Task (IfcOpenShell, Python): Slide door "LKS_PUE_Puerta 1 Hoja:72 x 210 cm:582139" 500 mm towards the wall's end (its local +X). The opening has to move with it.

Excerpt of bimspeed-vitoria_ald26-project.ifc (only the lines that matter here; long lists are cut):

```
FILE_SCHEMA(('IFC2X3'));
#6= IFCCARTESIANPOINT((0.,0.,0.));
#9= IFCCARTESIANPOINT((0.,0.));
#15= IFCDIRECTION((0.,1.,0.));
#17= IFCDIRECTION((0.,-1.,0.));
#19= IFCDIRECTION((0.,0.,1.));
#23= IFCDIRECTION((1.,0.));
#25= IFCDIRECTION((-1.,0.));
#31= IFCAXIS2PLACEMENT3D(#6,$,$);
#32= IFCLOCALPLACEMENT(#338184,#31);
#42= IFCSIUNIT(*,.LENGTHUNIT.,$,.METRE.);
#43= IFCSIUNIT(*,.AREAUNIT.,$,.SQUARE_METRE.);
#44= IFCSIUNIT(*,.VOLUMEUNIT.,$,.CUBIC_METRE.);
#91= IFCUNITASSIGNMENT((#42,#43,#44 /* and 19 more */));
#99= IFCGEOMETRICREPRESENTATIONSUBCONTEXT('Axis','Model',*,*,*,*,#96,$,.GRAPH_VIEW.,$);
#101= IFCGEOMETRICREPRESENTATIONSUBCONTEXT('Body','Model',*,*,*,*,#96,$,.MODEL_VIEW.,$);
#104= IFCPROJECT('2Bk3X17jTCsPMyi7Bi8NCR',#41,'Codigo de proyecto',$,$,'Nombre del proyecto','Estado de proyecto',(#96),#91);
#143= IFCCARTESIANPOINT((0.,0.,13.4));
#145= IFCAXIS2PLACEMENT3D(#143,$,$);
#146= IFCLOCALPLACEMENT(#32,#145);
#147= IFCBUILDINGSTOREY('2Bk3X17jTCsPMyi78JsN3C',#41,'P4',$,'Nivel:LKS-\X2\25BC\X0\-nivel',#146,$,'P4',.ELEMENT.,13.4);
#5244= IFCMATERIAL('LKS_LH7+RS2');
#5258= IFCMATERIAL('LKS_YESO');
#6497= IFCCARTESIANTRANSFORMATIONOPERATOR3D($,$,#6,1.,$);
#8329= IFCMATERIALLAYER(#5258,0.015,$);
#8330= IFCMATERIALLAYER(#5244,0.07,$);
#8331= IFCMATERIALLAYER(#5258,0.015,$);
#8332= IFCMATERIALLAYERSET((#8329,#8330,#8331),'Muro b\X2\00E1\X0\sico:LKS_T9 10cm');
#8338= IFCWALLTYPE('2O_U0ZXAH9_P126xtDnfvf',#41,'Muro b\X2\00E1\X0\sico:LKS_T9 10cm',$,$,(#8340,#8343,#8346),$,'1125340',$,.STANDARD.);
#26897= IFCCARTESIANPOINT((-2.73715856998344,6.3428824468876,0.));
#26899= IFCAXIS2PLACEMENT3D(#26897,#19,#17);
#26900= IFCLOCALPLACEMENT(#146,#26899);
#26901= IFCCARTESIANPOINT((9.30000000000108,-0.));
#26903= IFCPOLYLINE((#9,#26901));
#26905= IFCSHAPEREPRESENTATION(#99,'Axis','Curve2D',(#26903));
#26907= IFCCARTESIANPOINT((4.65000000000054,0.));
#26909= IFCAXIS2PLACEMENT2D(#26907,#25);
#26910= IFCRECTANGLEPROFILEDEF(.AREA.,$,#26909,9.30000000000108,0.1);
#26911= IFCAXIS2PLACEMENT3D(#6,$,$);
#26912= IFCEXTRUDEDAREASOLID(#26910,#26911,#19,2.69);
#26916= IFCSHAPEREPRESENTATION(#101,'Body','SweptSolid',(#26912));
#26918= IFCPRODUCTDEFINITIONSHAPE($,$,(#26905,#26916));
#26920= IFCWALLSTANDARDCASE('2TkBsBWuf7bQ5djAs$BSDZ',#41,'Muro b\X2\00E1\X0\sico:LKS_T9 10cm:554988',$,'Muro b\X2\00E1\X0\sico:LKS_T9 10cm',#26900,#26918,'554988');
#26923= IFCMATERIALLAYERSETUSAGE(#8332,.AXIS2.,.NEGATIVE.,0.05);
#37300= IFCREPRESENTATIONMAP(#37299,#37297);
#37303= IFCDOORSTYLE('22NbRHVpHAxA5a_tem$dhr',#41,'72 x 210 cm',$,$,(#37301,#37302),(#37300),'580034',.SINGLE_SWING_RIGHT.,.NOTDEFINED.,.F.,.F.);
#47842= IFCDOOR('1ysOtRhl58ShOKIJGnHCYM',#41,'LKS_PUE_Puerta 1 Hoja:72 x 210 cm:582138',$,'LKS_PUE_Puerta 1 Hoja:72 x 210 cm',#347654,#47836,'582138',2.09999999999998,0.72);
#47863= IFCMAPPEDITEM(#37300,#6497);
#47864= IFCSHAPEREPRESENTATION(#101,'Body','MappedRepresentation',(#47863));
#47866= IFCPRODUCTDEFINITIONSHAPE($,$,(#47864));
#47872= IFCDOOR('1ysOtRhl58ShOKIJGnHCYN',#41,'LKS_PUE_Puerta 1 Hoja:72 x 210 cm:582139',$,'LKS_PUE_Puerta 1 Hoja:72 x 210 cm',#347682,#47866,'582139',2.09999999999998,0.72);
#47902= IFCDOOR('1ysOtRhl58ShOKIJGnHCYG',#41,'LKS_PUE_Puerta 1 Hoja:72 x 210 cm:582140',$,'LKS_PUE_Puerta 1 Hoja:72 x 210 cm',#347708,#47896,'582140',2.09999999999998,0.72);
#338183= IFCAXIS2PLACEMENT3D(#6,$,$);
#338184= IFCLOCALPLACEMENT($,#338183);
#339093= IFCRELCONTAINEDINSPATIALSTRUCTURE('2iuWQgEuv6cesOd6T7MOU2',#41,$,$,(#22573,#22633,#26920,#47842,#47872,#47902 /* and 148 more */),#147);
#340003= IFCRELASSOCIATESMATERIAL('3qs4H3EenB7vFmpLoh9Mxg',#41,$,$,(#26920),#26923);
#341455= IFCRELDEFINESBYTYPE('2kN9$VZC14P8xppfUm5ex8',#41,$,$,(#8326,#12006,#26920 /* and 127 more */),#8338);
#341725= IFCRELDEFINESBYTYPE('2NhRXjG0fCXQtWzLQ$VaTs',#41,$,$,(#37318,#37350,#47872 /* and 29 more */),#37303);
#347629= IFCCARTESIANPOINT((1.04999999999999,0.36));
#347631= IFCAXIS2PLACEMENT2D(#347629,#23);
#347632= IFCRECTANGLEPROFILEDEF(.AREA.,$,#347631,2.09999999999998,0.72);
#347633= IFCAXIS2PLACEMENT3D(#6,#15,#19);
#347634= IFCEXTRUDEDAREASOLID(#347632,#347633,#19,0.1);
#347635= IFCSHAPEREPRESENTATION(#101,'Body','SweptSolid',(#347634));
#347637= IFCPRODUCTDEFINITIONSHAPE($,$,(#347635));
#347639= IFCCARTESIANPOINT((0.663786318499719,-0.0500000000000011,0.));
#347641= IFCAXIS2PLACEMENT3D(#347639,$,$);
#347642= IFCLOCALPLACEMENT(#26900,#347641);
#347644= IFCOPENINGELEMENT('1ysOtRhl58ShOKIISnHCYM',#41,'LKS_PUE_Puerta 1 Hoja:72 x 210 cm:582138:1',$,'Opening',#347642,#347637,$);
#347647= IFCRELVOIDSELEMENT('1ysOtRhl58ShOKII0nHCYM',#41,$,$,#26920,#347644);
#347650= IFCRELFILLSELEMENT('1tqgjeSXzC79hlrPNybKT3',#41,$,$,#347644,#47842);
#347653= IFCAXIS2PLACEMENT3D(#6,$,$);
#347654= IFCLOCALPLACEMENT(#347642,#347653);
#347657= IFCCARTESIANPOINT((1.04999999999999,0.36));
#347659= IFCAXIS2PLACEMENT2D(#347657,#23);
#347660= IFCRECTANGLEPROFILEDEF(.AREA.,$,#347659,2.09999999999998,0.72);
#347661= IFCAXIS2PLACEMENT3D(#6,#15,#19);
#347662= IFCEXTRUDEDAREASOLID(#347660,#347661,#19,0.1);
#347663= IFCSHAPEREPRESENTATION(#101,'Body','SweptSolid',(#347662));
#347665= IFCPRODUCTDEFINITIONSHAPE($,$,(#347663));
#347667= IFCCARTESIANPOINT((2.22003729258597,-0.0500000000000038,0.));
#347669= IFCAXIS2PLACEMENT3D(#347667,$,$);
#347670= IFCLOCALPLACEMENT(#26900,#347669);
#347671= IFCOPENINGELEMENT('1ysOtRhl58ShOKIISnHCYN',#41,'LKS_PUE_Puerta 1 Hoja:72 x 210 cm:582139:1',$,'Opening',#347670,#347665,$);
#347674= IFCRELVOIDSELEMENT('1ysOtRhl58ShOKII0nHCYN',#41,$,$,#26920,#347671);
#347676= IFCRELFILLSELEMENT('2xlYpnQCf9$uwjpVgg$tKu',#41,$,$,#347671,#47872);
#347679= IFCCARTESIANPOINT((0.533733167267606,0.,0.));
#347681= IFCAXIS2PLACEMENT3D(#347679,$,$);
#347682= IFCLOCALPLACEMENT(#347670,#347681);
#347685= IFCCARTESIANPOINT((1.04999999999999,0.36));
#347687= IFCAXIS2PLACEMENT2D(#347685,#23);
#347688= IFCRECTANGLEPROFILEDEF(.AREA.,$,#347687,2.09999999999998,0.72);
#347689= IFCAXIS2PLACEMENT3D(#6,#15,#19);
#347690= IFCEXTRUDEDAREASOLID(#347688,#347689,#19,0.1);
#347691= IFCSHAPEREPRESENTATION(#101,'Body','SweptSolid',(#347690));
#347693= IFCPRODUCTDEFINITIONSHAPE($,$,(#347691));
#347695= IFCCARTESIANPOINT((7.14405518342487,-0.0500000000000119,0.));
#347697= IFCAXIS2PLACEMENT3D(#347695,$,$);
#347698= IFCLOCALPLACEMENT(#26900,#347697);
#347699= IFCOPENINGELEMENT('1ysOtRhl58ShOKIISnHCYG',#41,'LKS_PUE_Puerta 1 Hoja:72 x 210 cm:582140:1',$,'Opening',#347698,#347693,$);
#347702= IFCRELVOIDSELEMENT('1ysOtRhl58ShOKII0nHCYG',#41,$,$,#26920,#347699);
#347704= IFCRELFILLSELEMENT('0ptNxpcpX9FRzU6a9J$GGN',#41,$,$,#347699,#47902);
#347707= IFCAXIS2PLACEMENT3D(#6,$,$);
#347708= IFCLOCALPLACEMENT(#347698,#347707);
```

```python
import ifcopenshell
import ifcopenshell.api.geometry
import ifcopenshell.util.placement
import ifcopenshell.util.unit

model = ifcopenshell.open("bimspeed-vitoria_ald26-project.ifc")
unit_scale = ifcopenshell.util.unit.calculate_unit_scale(model)

door = model.by_guid("1ysOtRhl58ShOKIJGnHCYN")
opening = door.FillsVoids[0].RelatingOpeningElement
wall = opening.VoidsElements[0].RelatingBuildingElement

wall_matrix = ifcopenshell.util.placement.get_local_placement(wall.ObjectPlacement)
shift = wall_matrix[:3, 0] * 0.5 / unit_scale
before = ifcopenshell.util.placement.get_local_placement(door.ObjectPlacement)[:3, 3].copy()

# The door is placed relative to its opening, so it follows when the opening moves.
matrix = ifcopenshell.util.placement.get_local_placement(opening.ObjectPlacement)
matrix[:3, 3] += shift
ifcopenshell.api.geometry.edit_object_placement(
    model, product=opening, matrix=matrix, is_si=False, should_transform_children=True
)

after = ifcopenshell.util.placement.get_local_placement(door.ObjectPlacement)[:3, 3]
print("door moved by", (after - before).round(3) + 0.0)

model.write("bimspeed-vitoria_ald26-project_v2.ifc")
```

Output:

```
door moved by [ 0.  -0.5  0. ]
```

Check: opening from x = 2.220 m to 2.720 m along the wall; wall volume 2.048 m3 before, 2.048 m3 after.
